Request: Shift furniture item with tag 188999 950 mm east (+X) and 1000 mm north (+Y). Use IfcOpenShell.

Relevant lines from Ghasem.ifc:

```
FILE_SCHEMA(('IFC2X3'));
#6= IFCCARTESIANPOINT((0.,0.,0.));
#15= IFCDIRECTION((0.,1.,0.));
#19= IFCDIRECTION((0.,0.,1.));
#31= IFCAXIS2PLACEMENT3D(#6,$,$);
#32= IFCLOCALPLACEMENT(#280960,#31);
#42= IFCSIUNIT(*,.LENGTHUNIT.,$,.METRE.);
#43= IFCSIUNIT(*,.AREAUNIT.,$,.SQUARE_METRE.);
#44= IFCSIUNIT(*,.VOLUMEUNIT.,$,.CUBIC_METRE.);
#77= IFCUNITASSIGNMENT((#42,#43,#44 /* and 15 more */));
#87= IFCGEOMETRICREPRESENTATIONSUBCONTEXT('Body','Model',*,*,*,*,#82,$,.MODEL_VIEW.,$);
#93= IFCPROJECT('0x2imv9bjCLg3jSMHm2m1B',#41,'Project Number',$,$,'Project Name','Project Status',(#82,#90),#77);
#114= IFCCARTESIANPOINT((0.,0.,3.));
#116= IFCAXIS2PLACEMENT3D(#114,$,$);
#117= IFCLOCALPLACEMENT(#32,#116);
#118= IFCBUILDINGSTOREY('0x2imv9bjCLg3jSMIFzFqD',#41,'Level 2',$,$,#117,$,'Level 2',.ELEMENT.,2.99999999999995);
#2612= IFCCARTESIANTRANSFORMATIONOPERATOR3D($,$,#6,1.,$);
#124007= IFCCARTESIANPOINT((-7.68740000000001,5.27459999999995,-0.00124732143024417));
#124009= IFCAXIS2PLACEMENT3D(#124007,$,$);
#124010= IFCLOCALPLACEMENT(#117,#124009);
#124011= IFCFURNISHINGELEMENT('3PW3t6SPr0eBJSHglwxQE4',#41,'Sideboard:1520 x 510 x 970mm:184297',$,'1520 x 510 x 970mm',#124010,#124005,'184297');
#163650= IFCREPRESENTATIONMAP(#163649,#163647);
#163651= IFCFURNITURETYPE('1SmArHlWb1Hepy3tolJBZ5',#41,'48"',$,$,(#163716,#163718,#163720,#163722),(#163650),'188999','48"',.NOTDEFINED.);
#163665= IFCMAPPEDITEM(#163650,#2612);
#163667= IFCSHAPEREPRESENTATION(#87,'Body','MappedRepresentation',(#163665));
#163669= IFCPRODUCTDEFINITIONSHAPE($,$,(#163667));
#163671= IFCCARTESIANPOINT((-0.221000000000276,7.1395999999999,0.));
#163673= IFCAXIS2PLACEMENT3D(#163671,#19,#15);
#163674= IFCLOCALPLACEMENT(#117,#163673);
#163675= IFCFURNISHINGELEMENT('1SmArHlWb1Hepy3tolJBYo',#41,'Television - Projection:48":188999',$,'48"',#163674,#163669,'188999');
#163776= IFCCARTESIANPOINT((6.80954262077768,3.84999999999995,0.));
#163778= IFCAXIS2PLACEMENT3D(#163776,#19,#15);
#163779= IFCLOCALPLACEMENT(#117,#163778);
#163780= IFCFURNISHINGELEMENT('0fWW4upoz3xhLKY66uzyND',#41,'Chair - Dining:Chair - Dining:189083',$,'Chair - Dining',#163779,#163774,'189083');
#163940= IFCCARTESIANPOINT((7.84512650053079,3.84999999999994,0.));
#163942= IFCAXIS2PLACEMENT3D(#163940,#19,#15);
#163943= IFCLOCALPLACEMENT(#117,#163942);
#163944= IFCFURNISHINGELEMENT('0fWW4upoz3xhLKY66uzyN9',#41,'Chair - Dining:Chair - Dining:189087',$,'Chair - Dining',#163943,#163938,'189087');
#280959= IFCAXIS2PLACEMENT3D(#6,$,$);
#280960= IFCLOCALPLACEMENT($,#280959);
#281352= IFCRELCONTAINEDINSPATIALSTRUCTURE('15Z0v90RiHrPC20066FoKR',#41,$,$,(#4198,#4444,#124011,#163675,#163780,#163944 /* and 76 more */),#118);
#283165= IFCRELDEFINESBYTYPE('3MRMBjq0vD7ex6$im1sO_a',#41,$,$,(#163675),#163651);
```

```python
import ifcopenshell
import ifcopenshell.api.geometry
import ifcopenshell.util.placement
import ifcopenshell.util.unit

model = ifcopenshell.open("Ghasem.ifc")
unit_scale = ifcopenshell.util.unit.calculate_unit_scale(model)

item = model.by_id(163675)
matrix = ifcopenshell.util.placement.get_local_placement(item.ObjectPlacement)
matrix[0, 3] += 0.95 / unit_scale
matrix[1, 3] += 1 / unit_scale
ifcopenshell.api.geometry.edit_object_placement(model, product=item, matrix=matrix, is_si=False)

print(ifcopenshell.util.placement.get_local_placement(item.ObjectPlacement).round(3) + 0.0)

model.write("Ghasem-out.ifc")
```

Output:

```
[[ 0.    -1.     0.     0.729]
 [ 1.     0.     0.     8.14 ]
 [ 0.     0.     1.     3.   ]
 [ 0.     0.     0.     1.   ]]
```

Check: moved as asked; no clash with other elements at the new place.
